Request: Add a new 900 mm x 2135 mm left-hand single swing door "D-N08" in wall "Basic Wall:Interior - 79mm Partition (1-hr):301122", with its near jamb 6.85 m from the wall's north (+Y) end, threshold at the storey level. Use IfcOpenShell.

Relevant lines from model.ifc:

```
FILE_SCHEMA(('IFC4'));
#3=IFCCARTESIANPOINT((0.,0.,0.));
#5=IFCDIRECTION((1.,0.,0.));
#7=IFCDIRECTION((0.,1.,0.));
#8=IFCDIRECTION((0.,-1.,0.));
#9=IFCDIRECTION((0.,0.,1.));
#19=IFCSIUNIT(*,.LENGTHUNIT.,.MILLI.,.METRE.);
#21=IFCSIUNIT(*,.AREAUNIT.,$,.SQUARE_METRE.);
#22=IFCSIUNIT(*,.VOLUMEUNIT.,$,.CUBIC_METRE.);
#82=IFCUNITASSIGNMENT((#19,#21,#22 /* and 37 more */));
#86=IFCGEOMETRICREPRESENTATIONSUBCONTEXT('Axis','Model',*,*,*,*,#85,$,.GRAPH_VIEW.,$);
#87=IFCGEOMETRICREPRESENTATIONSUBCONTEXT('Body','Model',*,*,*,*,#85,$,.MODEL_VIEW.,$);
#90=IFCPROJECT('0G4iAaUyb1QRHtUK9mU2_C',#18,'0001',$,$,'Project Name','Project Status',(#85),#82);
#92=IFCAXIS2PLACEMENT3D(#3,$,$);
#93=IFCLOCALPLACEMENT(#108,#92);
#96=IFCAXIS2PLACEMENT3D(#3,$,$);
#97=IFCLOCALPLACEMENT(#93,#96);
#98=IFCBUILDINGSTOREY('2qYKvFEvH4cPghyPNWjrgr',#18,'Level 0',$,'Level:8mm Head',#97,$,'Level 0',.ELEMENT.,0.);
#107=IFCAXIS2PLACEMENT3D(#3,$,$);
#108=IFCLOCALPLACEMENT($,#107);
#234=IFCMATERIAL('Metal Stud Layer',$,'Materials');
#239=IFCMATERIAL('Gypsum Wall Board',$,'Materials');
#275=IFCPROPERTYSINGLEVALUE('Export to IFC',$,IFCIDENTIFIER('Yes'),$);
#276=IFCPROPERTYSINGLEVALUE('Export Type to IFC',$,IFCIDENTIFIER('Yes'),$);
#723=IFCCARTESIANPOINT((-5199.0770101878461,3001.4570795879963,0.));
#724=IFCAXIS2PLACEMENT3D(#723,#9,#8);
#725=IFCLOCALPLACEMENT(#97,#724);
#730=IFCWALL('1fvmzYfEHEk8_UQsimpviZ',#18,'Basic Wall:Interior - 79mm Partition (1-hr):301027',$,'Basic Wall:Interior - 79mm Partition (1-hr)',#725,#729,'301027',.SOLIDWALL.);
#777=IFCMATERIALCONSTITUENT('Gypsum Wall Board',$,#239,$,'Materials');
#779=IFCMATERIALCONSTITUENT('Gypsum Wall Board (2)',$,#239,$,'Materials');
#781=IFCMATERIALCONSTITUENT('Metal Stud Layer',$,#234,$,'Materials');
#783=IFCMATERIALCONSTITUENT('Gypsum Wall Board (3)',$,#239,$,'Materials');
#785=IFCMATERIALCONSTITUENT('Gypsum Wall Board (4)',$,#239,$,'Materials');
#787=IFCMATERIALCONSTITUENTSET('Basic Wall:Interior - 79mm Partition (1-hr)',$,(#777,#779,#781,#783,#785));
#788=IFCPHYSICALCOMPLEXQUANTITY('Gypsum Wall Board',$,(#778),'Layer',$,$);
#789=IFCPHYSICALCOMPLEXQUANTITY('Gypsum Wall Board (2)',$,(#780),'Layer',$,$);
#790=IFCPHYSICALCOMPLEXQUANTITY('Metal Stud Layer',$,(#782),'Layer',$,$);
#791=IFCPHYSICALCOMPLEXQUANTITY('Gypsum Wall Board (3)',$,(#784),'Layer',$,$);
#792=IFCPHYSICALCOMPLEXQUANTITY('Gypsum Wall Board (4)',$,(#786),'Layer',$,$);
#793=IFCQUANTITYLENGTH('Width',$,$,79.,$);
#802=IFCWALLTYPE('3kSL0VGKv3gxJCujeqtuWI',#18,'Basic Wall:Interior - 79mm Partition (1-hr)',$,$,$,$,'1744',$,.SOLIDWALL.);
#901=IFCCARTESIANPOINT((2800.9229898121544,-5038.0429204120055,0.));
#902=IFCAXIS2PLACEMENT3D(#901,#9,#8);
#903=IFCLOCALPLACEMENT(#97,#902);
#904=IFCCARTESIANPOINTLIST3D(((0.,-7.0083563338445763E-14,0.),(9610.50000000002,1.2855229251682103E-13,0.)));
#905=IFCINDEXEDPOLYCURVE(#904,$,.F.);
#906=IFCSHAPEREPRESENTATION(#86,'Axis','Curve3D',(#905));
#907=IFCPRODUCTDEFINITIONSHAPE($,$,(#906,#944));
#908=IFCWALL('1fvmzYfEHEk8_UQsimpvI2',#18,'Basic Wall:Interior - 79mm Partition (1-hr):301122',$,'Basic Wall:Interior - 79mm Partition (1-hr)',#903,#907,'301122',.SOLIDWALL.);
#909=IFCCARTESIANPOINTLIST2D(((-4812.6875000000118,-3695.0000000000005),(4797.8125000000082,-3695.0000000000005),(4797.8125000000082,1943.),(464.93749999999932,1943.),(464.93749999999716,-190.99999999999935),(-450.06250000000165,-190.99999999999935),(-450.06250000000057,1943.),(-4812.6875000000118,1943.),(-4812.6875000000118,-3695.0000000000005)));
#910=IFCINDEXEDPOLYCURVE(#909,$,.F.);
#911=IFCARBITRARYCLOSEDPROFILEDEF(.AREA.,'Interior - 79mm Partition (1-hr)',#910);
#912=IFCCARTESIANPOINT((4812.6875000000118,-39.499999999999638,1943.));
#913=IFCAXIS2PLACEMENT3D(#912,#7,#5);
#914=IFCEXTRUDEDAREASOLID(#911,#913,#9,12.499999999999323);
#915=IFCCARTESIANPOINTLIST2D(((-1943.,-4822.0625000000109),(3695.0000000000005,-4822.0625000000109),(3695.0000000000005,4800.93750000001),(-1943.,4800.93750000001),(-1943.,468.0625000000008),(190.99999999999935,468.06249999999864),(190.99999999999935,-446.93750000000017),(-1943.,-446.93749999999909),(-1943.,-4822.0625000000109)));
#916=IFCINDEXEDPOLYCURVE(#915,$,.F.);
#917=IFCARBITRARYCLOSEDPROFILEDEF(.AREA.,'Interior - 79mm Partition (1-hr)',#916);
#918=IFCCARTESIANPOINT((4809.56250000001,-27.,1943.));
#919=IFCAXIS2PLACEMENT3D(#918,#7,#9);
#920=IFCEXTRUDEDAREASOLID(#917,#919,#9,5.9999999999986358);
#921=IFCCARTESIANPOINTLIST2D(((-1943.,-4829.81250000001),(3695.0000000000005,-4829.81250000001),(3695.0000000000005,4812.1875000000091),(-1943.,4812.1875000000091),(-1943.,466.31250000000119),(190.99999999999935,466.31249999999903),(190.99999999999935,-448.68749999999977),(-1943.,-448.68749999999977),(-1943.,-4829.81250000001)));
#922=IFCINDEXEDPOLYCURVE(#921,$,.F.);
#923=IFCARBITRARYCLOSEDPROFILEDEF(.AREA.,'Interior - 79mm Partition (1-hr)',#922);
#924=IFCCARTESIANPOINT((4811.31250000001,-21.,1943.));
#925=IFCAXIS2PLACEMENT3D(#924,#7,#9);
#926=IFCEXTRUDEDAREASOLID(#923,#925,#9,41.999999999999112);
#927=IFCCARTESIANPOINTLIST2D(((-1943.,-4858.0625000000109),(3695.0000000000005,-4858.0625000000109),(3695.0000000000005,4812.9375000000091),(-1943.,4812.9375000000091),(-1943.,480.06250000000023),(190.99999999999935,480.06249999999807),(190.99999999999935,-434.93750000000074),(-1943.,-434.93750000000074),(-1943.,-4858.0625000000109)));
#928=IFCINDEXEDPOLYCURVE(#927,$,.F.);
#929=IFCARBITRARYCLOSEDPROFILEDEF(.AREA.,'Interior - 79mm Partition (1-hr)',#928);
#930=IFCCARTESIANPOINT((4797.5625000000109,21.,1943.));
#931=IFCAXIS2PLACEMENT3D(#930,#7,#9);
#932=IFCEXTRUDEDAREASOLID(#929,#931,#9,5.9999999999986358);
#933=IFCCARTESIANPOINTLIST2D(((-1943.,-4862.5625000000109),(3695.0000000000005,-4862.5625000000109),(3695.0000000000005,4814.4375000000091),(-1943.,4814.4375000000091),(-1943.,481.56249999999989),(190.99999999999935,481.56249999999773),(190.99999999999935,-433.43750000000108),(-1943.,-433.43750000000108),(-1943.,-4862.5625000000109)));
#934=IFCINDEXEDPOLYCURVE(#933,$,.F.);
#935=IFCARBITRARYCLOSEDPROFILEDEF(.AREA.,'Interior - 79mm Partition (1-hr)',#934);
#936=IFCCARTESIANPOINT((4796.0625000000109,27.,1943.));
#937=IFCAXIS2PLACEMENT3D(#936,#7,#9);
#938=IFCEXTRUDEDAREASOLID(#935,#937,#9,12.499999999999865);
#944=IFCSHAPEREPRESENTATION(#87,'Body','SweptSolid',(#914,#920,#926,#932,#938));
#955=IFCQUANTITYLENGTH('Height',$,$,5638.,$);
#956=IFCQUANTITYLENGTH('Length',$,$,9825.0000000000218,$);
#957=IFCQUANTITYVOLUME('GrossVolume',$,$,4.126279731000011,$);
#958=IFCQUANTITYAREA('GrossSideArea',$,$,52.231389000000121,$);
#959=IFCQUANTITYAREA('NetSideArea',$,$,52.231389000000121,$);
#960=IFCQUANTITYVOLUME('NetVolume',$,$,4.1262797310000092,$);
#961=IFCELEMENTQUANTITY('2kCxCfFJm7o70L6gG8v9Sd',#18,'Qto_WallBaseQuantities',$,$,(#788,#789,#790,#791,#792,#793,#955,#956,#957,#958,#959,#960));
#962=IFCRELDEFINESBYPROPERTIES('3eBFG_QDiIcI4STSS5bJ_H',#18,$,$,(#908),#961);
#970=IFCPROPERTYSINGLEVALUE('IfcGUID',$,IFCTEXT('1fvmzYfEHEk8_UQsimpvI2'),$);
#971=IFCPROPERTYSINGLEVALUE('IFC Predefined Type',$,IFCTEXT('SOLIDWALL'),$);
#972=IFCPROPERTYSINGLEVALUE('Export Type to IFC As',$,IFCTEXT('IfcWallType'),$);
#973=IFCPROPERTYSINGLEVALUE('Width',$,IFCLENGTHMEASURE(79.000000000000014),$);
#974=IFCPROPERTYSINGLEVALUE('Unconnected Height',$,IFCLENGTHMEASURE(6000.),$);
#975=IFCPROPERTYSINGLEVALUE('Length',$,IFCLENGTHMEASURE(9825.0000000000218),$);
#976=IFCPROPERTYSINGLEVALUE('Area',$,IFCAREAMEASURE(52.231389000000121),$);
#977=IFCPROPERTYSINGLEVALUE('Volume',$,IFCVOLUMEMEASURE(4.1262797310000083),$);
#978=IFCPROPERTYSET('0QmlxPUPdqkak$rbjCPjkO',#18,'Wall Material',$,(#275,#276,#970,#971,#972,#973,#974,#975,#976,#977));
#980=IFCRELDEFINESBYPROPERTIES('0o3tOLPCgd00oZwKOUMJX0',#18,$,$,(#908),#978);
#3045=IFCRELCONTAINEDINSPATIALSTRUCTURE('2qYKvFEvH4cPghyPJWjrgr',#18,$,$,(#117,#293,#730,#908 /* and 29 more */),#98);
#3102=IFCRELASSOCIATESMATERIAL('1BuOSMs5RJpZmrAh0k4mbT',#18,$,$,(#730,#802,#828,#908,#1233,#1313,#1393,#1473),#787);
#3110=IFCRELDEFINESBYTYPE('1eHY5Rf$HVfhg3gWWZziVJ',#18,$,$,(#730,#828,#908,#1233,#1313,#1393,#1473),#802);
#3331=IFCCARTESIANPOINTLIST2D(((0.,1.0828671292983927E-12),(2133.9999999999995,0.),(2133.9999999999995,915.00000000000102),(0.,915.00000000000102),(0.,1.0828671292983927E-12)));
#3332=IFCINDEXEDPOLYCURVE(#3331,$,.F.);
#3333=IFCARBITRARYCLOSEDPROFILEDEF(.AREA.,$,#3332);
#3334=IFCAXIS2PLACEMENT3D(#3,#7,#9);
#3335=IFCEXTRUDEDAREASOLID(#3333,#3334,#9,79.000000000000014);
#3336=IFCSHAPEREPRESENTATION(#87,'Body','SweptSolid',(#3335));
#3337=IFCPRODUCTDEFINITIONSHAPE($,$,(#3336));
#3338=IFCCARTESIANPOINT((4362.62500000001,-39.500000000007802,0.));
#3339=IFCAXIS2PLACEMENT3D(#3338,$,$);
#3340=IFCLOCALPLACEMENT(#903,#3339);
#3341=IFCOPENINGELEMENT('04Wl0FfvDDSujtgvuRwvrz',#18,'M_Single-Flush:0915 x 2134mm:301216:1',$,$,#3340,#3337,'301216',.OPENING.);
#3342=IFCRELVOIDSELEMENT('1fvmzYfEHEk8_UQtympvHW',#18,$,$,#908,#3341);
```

```python
import numpy as np
import ifcopenshell
import ifcopenshell.api.feature
import ifcopenshell.api.geometry
import ifcopenshell.api.pset
import ifcopenshell.api.root
import ifcopenshell.api.spatial
import ifcopenshell.geom
import ifcopenshell.util.element
import ifcopenshell.util.placement
import ifcopenshell.util.representation
import ifcopenshell.util.shape
import ifcopenshell.util.unit

model = ifcopenshell.open("model.ifc")
unit_scale = ifcopenshell.util.unit.calculate_unit_scale(model)
area_scale = ifcopenshell.util.unit.calculate_unit_scale(model, "AREAUNIT")
volume_scale = ifcopenshell.util.unit.calculate_unit_scale(model, "VOLUMEUNIT")
settings = ifcopenshell.geom.settings()


def volume(element):
    """Net volume in cubic metres, openings subtracted."""
    shape = ifcopenshell.geom.create_shape(settings, element)
    return ifcopenshell.util.shape.get_volume(shape.geometry)


wall = model.by_guid("1fvmzYfEHEk8_UQsimpvI2")
storey = ifcopenshell.util.element.get_container(wall, ifc_class="IfcBuildingStorey")
context = ifcopenshell.util.representation.get_context(model, "Model", "Body", "MODEL_VIEW")
before = volume(wall)

width, height, from_end, sill = 0.9, 2.135, 6.85, 0.0  # metres

# The wall runs along its own X axis, and the end named is its -X end.
wall_shape = ifcopenshell.geom.create_shape(settings, wall)
x, y, z = ifcopenshell.util.shape.get_vertices(wall_shape.geometry).T
start = x.min() + from_end
face, thickness = float(y.min()), float(y.max() - y.min())
wall_matrix = ifcopenshell.util.placement.get_local_placement(wall.ObjectPlacement)
level = ifcopenshell.util.placement.get_local_placement(storey.ObjectPlacement)[2, 3]


def in_wall(x, y):
    """Placement at x, y metres in the wall's axes, at sill height."""
    matrix = wall_matrix.copy()
    matrix[:, 3] = wall_matrix @ np.array([x / unit_scale, y / unit_scale, 0.0, 1.0])
    matrix[2, 3] = level + sill / unit_scale
    return matrix


# Opening: a box that overshoots both wall faces by 50 mm.
opening = ifcopenshell.api.root.create_entity(model, ifc_class="IfcOpeningElement", predefined_type="OPENING")
box = ifcopenshell.api.geometry.add_wall_representation(
    model, context=context, length=width, height=height, thickness=thickness + 0.1
)
ifcopenshell.api.geometry.assign_representation(model, product=opening, representation=box)
ifcopenshell.api.geometry.edit_object_placement(model, product=opening, matrix=in_wall(start, face - 0.05), is_si=False)
ifcopenshell.api.feature.add_feature(model, feature=opening, element=wall)

door = ifcopenshell.api.root.create_entity(model, ifc_class="IfcDoor", name="D-N08", predefined_type="DOOR")
door.OverallWidth, door.OverallHeight = width / unit_scale, height / unit_scale
door.OperationType = "SINGLE_SWING_LEFT"
body = ifcopenshell.api.geometry.add_door_representation(
    model,
    context=context,
    overall_width=door.OverallWidth,
    overall_height=door.OverallHeight,
    operation_type="SINGLE_SWING_LEFT",
    lining_properties={"LiningDepth": thickness / unit_scale, "ThresholdDepth": thickness / unit_scale},
)
ifcopenshell.api.geometry.assign_representation(model, product=door, representation=body)
ifcopenshell.api.spatial.assign_container(model, products=[door], relating_structure=storey)
ifcopenshell.api.feature.add_filling(model, opening=opening, element=door)

# The lining spans the wall, so the door starts at the wall face.
ifcopenshell.api.geometry.edit_object_placement(model, product=door, matrix=in_wall(start, face), is_si=False)

after = volume(wall)

# Update the wall's stored quantities.
qto = model.by_id(ifcopenshell.util.element.get_pset(wall, "Qto_WallBaseQuantities", should_inherit=False)["id"])
ifcopenshell.api.pset.edit_qto(model, qto=qto, properties={
    "NetSideArea": after / thickness / area_scale,
    "NetVolume": after / volume_scale,
})
pset = model.by_id(ifcopenshell.util.element.get_pset(wall, "Wall Material", should_inherit=False)["id"])
ifcopenshell.api.pset.edit_pset(model, pset=pset, properties={
    "Area": model.create_entity("IfcAreaMeasure", after / thickness / area_scale),
    "Volume": model.create_entity("IfcVolumeMeasure", after / volume_scale),
})

print(f"wall volume {before:.3f} -> {after:.3f} m3")

model.write("model_rev.ifc")
```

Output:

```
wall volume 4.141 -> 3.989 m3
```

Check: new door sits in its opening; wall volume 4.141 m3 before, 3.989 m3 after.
